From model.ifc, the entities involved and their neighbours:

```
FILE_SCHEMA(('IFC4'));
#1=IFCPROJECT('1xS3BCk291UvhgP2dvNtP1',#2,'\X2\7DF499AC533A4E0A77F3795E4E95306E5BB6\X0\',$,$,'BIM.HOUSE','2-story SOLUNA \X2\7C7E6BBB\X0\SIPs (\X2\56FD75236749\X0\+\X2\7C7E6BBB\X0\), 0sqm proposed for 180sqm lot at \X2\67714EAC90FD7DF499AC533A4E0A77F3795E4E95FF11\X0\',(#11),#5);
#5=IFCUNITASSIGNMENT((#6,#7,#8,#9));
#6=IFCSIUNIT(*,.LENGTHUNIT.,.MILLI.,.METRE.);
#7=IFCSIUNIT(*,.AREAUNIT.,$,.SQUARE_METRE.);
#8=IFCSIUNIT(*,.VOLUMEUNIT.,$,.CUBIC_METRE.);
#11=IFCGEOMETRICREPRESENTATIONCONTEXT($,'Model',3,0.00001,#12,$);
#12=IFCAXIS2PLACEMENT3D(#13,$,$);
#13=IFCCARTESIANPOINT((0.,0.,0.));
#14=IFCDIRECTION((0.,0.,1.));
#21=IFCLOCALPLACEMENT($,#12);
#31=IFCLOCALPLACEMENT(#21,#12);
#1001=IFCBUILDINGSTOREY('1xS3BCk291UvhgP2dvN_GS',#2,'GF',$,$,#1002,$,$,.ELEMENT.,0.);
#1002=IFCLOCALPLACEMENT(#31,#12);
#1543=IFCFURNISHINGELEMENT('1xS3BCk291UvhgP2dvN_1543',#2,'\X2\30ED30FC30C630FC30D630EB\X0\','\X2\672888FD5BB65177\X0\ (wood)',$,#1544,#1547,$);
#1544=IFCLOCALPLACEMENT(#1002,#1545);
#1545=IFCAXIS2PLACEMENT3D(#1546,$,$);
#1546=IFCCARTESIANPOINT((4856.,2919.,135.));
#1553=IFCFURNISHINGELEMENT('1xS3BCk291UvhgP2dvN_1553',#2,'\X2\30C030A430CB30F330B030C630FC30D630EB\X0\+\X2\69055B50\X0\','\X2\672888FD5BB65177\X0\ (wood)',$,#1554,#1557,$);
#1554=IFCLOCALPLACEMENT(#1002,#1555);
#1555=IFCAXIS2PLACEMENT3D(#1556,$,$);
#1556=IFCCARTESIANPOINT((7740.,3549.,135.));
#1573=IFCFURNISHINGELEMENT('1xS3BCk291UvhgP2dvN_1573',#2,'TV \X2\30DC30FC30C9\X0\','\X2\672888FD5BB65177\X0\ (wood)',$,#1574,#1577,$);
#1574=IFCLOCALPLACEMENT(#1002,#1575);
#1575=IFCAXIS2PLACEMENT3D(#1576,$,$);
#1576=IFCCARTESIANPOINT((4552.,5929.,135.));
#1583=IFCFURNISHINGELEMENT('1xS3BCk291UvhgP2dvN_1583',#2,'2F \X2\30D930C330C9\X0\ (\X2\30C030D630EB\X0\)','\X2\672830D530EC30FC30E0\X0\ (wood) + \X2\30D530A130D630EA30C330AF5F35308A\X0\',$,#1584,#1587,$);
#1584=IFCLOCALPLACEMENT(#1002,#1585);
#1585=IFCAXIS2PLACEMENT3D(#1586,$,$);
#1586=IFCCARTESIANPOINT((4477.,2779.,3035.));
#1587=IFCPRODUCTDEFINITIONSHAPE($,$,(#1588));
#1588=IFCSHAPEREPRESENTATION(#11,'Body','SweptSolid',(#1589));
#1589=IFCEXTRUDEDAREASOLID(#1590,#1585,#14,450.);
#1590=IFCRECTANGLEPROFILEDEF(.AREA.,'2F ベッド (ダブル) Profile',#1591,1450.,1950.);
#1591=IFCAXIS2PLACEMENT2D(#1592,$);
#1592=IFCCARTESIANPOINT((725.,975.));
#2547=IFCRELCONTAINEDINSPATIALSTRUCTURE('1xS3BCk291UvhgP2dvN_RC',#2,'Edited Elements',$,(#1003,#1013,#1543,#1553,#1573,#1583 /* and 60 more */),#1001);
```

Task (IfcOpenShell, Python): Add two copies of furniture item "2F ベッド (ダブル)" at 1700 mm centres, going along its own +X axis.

```python
import ifcopenshell
import ifcopenshell.api.geometry
import ifcopenshell.api.root
import ifcopenshell.util.element
import ifcopenshell.util.placement
import ifcopenshell.util.unit

model = ifcopenshell.open("model.ifc")
unit_scale = ifcopenshell.util.unit.calculate_unit_scale(model)


def reuse_history(source, copy):
    """copy_class also copies each property set's owner history, people and application; keep the originals."""
    for rel in copy.IsDefinedBy:
        if rel.is_a("IfcRelDefinesByProperties") and (history := rel.RelatingPropertyDefinition.OwnerHistory):
            rel.RelatingPropertyDefinition.OwnerHistory = source.OwnerHistory
            ifcopenshell.util.element.remove_deep2(model, history)


source = model.by_guid("1xS3BCk291UvhgP2dvN_1583")
base = ifcopenshell.util.placement.get_local_placement(source.ObjectPlacement)
step = base[:3, 0] * 1.7 / unit_scale

for i in range(1, 3):
    copy = ifcopenshell.api.root.copy_class(model, product=source)
    copy.Representation = ifcopenshell.util.element.copy_deep(
        model, source.Representation, exclude=["IfcGeometricRepresentationContext", "IfcRepresentationMap"]
    )
    reuse_history(source, copy)
    matrix = base.copy()
    matrix[:3, 3] += i * step
    print("added at", matrix[:3, 3].round(3) + 0.0)
    ifcopenshell.api.geometry.edit_object_placement(model, product=copy, matrix=matrix, is_si=False)

model.write("model_v2.ifc")
```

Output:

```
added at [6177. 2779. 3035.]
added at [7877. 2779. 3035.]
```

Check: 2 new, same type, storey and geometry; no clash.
